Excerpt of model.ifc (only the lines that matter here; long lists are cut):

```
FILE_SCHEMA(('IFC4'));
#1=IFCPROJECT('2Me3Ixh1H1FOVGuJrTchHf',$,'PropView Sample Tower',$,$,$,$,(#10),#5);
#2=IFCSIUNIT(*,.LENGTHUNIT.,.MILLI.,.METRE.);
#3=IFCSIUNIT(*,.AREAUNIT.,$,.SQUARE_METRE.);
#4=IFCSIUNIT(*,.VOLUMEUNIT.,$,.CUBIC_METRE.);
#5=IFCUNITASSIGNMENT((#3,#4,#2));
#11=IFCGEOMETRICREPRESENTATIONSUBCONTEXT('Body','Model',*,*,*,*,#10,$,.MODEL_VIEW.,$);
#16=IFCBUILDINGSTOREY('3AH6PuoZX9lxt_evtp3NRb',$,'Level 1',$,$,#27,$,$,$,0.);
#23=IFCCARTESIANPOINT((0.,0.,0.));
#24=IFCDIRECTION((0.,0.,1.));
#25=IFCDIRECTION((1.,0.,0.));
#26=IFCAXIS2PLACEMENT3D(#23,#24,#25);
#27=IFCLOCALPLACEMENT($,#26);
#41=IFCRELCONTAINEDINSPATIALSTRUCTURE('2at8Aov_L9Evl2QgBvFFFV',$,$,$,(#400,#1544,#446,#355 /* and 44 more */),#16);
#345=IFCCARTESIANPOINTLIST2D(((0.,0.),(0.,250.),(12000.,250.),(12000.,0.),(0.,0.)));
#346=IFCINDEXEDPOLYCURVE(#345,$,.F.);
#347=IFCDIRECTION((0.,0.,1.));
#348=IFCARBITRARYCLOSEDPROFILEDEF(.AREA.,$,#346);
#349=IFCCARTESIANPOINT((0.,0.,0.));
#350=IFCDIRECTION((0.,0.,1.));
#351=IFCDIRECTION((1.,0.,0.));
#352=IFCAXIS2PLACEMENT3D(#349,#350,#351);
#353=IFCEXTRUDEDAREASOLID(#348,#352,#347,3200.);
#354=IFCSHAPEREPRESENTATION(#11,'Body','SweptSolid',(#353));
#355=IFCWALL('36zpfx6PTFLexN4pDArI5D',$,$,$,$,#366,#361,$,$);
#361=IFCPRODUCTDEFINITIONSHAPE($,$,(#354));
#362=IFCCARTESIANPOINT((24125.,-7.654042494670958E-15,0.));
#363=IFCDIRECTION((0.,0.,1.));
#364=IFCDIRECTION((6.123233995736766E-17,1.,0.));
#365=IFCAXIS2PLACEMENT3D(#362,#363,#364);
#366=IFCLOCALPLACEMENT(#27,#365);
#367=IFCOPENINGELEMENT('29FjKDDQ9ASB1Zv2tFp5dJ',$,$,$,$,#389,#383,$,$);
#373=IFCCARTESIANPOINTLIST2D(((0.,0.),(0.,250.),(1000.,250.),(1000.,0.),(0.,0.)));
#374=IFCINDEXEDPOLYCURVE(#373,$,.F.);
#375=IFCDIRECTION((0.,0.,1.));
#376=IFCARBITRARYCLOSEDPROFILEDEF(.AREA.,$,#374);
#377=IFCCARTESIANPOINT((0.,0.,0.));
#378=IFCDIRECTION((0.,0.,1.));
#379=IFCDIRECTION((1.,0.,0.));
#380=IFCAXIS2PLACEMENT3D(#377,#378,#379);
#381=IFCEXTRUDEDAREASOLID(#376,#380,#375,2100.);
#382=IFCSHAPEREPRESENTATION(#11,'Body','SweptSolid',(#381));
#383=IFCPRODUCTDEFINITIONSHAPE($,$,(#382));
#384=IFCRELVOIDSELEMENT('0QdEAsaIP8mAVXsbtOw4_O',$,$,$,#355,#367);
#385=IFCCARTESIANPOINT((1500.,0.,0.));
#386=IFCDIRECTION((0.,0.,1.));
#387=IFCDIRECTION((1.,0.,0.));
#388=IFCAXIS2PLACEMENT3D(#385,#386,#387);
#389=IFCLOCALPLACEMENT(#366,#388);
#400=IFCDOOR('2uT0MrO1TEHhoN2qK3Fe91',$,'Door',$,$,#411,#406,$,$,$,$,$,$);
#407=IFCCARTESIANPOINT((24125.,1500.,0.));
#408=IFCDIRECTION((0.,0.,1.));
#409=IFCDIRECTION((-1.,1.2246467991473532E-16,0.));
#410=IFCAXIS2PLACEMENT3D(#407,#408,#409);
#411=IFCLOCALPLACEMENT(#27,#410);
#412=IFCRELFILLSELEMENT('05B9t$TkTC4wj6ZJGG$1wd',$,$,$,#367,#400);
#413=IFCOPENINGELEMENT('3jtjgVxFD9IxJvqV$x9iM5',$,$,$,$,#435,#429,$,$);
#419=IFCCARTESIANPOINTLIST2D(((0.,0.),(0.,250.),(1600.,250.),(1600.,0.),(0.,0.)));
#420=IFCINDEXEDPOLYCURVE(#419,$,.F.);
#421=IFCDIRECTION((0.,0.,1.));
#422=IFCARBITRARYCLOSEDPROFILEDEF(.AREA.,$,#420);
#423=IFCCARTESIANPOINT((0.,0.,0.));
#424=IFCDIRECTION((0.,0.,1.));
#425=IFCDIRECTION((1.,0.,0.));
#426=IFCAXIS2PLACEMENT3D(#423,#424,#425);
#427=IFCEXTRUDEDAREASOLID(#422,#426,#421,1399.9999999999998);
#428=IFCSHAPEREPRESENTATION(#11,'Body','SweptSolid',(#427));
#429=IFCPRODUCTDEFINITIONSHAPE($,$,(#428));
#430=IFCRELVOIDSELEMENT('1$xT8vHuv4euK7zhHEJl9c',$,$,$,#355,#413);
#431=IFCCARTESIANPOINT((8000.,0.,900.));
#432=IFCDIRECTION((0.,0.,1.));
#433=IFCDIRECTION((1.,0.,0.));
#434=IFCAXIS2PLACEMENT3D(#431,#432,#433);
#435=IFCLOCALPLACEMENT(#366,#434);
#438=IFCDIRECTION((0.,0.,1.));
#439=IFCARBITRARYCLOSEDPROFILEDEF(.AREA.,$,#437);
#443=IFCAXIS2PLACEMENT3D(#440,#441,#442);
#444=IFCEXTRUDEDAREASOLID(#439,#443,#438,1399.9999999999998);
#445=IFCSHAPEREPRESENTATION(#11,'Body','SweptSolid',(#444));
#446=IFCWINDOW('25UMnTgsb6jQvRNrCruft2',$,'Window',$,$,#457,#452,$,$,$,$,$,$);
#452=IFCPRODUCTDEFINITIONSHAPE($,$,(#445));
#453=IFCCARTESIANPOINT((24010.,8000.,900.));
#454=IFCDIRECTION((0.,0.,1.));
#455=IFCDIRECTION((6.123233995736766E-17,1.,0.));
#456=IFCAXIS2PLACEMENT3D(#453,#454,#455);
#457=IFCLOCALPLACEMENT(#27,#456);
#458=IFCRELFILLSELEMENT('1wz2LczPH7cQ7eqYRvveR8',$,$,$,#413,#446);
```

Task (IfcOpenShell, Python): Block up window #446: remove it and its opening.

```python
import ifcopenshell
import ifcopenshell.api.feature
import ifcopenshell.api.root
import ifcopenshell.geom
import ifcopenshell.util.shape

model = ifcopenshell.open("model.ifc")
settings = ifcopenshell.geom.settings()


def volume(element):
    """Net volume in cubic metres, openings subtracted."""
    shape = ifcopenshell.geom.create_shape(settings, element)
    return ifcopenshell.util.shape.get_volume(shape.geometry)


window = model.by_guid("25UMnTgsb6jQvRNrCruft2")
opening = window.FillsVoids[0].RelatingOpeningElement
wall = opening.VoidsElements[0].RelatingBuildingElement
before = volume(wall)

ifcopenshell.api.root.remove_product(model, product=window)
ifcopenshell.api.feature.remove_feature(model, feature=opening)

after = volume(wall)

print(f"wall volume {before:.3f} -> {after:.3f} m3")

model.write("model-out.ifc")
```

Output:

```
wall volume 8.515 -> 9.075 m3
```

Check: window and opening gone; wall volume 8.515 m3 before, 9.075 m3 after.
